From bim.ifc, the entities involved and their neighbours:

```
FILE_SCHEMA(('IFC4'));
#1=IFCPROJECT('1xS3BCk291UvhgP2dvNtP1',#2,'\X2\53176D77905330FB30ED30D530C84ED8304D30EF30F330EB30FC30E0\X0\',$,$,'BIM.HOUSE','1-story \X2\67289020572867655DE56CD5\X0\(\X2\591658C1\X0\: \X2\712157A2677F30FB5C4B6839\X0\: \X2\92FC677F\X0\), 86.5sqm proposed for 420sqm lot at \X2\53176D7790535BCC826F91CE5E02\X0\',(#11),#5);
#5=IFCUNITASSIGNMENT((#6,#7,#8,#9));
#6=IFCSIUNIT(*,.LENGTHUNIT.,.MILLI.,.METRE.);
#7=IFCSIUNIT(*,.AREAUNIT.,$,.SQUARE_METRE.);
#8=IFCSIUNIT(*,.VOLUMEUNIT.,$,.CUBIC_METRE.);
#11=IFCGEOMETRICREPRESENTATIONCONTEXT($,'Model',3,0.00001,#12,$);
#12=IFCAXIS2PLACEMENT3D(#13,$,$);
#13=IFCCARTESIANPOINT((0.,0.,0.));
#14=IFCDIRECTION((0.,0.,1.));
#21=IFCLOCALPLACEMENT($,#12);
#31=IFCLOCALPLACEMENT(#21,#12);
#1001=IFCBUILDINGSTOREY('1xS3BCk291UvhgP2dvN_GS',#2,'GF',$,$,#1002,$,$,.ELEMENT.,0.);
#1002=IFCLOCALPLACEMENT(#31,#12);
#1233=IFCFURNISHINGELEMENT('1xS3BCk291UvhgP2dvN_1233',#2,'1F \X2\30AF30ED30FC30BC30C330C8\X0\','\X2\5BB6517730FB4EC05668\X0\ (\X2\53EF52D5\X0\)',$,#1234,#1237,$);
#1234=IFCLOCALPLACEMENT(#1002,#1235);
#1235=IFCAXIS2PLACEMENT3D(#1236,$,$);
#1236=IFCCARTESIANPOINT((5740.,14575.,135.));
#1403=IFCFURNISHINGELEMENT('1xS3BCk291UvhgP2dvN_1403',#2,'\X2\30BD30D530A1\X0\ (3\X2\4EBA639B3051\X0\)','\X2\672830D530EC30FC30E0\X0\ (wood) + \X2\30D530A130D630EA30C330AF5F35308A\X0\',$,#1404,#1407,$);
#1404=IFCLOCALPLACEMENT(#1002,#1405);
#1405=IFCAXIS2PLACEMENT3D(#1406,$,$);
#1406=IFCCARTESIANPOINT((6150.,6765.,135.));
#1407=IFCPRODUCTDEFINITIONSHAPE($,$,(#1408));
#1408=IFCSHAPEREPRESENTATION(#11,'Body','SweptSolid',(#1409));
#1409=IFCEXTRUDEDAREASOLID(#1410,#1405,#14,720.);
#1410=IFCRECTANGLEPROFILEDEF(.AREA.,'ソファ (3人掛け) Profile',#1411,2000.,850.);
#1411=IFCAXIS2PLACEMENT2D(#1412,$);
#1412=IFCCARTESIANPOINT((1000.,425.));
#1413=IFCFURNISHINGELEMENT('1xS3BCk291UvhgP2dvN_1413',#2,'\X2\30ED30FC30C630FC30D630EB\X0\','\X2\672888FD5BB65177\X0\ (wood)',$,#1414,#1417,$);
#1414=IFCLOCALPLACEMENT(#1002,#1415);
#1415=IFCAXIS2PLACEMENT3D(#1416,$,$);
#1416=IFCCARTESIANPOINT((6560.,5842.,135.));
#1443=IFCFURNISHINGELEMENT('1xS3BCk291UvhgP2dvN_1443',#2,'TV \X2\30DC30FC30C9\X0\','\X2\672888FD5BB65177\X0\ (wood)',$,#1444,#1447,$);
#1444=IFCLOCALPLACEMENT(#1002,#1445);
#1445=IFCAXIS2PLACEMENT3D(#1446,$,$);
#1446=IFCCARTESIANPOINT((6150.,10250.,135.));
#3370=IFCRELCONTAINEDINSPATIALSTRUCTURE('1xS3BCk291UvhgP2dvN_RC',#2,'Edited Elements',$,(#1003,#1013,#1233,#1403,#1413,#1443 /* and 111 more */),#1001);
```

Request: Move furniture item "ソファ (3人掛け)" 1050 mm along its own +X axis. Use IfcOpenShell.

```python
import ifcopenshell
import ifcopenshell.api.geometry
import ifcopenshell.util.placement

model = ifcopenshell.open("bim.ifc")

item = model.by_guid("1xS3BCk291UvhgP2dvN_1403")
matrix = ifcopenshell.util.placement.get_local_placement(item.ObjectPlacement)
matrix[:3, 3] += matrix[:3, 0] * 1050.0
ifcopenshell.api.geometry.edit_object_placement(model, product=item, matrix=matrix, is_si=False)

print(ifcopenshell.util.placement.get_local_placement(item.ObjectPlacement).round(3) + 0.0)

model.write("bim-out.ifc")
```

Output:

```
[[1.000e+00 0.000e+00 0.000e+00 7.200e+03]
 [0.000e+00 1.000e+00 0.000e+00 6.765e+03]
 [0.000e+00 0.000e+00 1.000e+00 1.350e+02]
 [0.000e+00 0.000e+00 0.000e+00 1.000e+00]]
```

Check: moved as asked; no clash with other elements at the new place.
